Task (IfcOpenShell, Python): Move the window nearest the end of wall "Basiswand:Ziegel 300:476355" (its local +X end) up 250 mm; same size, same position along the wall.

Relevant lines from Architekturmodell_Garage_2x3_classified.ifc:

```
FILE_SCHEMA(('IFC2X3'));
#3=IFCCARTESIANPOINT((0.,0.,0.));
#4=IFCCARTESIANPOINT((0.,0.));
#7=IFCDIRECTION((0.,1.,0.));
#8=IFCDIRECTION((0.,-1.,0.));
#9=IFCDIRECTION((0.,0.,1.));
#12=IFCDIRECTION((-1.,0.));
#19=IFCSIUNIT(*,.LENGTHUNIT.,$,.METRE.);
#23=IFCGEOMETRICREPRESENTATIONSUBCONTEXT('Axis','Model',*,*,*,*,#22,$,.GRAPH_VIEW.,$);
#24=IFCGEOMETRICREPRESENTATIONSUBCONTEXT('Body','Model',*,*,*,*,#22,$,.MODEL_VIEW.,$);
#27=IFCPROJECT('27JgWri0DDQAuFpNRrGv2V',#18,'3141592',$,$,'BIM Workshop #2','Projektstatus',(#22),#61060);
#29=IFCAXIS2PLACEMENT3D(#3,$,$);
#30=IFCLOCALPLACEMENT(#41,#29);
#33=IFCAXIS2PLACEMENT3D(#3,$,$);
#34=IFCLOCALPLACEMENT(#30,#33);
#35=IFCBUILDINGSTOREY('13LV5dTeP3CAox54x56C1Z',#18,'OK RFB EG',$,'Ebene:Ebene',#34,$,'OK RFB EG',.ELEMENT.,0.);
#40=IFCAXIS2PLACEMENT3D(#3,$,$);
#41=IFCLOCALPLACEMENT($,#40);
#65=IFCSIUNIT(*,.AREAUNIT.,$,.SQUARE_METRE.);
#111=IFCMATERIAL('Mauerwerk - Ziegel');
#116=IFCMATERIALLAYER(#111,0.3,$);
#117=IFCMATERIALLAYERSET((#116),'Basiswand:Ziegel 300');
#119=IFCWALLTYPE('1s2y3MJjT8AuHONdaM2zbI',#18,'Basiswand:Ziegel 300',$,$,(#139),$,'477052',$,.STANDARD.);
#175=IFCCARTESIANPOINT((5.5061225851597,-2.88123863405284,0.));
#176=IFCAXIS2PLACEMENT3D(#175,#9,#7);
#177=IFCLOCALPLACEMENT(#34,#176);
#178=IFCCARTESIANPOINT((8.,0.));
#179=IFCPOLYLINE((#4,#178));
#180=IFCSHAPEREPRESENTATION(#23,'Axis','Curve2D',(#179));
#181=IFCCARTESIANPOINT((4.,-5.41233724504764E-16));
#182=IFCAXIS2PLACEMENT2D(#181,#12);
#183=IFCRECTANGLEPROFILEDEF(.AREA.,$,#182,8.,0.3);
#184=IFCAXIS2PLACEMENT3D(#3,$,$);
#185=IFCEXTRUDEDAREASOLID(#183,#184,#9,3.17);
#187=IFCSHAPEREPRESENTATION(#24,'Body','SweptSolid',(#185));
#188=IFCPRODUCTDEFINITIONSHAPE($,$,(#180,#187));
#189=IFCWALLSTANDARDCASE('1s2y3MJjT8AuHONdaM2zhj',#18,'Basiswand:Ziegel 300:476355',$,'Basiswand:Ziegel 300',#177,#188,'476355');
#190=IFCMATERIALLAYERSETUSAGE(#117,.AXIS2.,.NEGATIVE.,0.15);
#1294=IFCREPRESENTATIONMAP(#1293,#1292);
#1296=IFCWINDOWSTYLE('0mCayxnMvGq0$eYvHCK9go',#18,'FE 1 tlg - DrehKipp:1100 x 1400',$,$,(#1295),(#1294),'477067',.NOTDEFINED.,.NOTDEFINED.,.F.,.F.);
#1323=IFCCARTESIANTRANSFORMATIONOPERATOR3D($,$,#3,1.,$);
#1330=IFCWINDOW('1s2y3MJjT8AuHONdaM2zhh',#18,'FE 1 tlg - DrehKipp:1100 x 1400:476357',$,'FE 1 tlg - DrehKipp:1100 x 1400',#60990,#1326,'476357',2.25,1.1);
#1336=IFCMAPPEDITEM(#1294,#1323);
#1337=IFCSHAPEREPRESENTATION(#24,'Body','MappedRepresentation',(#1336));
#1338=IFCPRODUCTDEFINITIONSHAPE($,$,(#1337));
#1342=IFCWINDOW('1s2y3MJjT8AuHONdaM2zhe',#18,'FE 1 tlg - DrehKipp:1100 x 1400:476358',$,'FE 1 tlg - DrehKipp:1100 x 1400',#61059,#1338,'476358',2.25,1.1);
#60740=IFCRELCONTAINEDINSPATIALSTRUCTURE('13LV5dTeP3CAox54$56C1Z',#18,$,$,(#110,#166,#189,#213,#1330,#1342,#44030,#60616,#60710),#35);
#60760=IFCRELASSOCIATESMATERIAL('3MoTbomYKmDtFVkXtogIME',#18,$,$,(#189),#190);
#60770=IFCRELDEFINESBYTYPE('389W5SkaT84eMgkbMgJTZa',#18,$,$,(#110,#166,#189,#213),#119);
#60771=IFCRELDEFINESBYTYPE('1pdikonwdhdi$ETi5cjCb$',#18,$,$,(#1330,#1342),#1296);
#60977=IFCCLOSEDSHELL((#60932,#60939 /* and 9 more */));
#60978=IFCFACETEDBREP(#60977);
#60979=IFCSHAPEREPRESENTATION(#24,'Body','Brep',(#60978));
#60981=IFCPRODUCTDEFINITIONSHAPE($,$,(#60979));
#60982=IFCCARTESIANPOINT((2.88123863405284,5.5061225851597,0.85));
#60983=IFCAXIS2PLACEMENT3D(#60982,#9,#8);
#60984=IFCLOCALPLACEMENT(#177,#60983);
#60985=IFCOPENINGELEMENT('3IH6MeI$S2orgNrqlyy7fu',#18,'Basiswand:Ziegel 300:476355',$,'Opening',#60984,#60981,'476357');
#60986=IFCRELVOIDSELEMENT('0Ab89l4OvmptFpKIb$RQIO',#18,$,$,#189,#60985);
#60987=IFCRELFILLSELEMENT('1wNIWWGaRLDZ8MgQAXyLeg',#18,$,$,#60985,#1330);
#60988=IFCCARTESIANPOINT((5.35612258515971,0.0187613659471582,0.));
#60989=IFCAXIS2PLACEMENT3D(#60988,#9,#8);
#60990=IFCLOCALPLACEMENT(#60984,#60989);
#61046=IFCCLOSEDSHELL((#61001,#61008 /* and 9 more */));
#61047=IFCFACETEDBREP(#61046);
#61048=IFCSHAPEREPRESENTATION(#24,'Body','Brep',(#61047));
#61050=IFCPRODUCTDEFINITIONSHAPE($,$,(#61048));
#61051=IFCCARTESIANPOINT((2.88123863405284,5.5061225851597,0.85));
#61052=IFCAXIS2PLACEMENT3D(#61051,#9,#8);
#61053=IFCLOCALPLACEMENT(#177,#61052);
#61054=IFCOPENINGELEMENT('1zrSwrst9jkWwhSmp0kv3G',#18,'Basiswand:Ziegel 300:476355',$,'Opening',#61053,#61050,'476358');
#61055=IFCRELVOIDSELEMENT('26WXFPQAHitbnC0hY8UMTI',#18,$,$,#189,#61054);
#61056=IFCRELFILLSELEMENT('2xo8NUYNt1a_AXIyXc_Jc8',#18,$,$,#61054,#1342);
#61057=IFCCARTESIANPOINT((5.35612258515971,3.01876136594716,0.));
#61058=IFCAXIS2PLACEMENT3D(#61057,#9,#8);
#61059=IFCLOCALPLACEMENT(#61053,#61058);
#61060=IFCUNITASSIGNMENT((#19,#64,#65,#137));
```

```python
import numpy as np
import ifcopenshell
import ifcopenshell.api.geometry
import ifcopenshell.util.placement
import ifcopenshell.util.unit

model = ifcopenshell.open("Architekturmodell_Garage_2x3_classified.ifc")
unit_scale = ifcopenshell.util.unit.calculate_unit_scale(model)

window = model.by_guid("1s2y3MJjT8AuHONdaM2zhe")
opening = window.FillsVoids[0].RelatingOpeningElement
dz = 0.25

shift = np.array([0.0, 0.0, dz])
# The window is placed relative to its opening, so it follows when the opening moves.
matrix = ifcopenshell.util.placement.get_local_placement(opening.ObjectPlacement)
matrix[:3, 3] += shift
ifcopenshell.api.geometry.edit_object_placement(
    model, product=opening, matrix=matrix, is_si=False, should_transform_children=True
)

print(f"moved by {dz * unit_scale:+.3f} m")

model.write("Architekturmodell_Garage_2x3_classified_v2.ifc")
```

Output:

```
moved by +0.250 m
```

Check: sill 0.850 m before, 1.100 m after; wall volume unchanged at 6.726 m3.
